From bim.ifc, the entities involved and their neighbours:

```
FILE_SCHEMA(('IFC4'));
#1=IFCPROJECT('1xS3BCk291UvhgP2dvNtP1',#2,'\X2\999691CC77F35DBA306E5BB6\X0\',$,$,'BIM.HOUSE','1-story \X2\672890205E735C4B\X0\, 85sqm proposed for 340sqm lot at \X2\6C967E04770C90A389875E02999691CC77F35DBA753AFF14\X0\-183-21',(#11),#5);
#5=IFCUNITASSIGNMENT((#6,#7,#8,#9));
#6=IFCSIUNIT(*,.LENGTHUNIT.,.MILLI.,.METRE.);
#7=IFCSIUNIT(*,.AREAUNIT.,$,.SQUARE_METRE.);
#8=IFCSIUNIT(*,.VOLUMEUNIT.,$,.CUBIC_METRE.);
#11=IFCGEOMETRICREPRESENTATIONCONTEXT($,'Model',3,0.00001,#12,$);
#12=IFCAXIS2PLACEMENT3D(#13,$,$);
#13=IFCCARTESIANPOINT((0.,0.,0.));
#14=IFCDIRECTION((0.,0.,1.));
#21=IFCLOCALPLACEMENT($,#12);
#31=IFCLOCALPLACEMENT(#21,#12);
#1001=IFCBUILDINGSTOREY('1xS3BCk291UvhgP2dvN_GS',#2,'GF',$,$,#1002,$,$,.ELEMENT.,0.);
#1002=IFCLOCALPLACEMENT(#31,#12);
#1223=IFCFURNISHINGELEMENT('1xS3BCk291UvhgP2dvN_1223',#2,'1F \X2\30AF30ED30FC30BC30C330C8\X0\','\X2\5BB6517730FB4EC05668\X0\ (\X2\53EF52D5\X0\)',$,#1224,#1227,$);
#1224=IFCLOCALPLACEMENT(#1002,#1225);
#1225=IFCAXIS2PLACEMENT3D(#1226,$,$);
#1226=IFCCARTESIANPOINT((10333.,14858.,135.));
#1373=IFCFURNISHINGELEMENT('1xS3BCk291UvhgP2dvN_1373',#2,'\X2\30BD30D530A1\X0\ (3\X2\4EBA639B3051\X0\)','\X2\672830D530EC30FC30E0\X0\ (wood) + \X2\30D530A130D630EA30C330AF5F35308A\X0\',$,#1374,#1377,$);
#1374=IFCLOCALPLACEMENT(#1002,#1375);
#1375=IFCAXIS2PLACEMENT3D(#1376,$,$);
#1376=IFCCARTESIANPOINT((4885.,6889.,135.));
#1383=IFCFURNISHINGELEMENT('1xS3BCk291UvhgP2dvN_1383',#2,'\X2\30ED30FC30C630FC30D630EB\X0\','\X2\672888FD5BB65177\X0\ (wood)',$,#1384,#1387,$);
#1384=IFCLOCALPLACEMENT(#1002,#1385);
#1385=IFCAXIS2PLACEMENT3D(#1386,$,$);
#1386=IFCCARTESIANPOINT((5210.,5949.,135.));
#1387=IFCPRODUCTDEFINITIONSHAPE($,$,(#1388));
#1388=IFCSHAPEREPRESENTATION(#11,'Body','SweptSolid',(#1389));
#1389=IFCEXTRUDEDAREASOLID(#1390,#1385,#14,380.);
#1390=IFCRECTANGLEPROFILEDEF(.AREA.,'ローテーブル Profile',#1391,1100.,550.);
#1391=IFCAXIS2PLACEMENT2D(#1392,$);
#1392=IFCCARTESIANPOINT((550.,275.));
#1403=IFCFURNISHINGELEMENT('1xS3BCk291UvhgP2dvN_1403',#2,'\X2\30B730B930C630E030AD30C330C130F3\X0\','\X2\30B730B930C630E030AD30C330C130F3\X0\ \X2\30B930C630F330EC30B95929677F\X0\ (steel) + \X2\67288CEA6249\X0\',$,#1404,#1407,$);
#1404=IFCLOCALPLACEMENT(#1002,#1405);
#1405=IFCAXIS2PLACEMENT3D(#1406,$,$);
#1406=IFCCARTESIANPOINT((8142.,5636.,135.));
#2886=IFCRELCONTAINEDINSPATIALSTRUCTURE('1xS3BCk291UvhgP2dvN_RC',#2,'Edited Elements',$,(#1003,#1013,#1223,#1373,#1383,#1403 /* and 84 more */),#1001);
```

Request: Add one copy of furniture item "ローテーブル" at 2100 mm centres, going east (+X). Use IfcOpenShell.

```python
import numpy as np
import ifcopenshell
import ifcopenshell.api.geometry
import ifcopenshell.api.root
import ifcopenshell.util.element
import ifcopenshell.util.placement
import ifcopenshell.util.unit

model = ifcopenshell.open("bim.ifc")
unit_scale = ifcopenshell.util.unit.calculate_unit_scale(model)


def reuse_history(source, copy):
    """copy_class also copies each property set's owner history, people and application; keep the originals."""
    for rel in copy.IsDefinedBy:
        if rel.is_a("IfcRelDefinesByProperties") and (history := rel.RelatingPropertyDefinition.OwnerHistory):
            rel.RelatingPropertyDefinition.OwnerHistory = source.OwnerHistory
            ifcopenshell.util.element.remove_deep2(model, history)


source = model.by_guid("1xS3BCk291UvhgP2dvN_1383")
base = ifcopenshell.util.placement.get_local_placement(source.ObjectPlacement)
step = np.array([1.0, 0.0, 0.0]) * 2.1 / unit_scale

for i in range(1, 2):
    copy = ifcopenshell.api.root.copy_class(model, product=source)
    copy.Representation = ifcopenshell.util.element.copy_deep(
        model, source.Representation, exclude=["IfcGeometricRepresentationContext", "IfcRepresentationMap"]
    )
    reuse_history(source, copy)
    matrix = base.copy()
    matrix[:3, 3] += i * step
    print("added at", matrix[:3, 3].round(3) + 0.0)
    ifcopenshell.api.geometry.edit_object_placement(model, product=copy, matrix=matrix, is_si=False)

model.write("bim_edited.ifc")
```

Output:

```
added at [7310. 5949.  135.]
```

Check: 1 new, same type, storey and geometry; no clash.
